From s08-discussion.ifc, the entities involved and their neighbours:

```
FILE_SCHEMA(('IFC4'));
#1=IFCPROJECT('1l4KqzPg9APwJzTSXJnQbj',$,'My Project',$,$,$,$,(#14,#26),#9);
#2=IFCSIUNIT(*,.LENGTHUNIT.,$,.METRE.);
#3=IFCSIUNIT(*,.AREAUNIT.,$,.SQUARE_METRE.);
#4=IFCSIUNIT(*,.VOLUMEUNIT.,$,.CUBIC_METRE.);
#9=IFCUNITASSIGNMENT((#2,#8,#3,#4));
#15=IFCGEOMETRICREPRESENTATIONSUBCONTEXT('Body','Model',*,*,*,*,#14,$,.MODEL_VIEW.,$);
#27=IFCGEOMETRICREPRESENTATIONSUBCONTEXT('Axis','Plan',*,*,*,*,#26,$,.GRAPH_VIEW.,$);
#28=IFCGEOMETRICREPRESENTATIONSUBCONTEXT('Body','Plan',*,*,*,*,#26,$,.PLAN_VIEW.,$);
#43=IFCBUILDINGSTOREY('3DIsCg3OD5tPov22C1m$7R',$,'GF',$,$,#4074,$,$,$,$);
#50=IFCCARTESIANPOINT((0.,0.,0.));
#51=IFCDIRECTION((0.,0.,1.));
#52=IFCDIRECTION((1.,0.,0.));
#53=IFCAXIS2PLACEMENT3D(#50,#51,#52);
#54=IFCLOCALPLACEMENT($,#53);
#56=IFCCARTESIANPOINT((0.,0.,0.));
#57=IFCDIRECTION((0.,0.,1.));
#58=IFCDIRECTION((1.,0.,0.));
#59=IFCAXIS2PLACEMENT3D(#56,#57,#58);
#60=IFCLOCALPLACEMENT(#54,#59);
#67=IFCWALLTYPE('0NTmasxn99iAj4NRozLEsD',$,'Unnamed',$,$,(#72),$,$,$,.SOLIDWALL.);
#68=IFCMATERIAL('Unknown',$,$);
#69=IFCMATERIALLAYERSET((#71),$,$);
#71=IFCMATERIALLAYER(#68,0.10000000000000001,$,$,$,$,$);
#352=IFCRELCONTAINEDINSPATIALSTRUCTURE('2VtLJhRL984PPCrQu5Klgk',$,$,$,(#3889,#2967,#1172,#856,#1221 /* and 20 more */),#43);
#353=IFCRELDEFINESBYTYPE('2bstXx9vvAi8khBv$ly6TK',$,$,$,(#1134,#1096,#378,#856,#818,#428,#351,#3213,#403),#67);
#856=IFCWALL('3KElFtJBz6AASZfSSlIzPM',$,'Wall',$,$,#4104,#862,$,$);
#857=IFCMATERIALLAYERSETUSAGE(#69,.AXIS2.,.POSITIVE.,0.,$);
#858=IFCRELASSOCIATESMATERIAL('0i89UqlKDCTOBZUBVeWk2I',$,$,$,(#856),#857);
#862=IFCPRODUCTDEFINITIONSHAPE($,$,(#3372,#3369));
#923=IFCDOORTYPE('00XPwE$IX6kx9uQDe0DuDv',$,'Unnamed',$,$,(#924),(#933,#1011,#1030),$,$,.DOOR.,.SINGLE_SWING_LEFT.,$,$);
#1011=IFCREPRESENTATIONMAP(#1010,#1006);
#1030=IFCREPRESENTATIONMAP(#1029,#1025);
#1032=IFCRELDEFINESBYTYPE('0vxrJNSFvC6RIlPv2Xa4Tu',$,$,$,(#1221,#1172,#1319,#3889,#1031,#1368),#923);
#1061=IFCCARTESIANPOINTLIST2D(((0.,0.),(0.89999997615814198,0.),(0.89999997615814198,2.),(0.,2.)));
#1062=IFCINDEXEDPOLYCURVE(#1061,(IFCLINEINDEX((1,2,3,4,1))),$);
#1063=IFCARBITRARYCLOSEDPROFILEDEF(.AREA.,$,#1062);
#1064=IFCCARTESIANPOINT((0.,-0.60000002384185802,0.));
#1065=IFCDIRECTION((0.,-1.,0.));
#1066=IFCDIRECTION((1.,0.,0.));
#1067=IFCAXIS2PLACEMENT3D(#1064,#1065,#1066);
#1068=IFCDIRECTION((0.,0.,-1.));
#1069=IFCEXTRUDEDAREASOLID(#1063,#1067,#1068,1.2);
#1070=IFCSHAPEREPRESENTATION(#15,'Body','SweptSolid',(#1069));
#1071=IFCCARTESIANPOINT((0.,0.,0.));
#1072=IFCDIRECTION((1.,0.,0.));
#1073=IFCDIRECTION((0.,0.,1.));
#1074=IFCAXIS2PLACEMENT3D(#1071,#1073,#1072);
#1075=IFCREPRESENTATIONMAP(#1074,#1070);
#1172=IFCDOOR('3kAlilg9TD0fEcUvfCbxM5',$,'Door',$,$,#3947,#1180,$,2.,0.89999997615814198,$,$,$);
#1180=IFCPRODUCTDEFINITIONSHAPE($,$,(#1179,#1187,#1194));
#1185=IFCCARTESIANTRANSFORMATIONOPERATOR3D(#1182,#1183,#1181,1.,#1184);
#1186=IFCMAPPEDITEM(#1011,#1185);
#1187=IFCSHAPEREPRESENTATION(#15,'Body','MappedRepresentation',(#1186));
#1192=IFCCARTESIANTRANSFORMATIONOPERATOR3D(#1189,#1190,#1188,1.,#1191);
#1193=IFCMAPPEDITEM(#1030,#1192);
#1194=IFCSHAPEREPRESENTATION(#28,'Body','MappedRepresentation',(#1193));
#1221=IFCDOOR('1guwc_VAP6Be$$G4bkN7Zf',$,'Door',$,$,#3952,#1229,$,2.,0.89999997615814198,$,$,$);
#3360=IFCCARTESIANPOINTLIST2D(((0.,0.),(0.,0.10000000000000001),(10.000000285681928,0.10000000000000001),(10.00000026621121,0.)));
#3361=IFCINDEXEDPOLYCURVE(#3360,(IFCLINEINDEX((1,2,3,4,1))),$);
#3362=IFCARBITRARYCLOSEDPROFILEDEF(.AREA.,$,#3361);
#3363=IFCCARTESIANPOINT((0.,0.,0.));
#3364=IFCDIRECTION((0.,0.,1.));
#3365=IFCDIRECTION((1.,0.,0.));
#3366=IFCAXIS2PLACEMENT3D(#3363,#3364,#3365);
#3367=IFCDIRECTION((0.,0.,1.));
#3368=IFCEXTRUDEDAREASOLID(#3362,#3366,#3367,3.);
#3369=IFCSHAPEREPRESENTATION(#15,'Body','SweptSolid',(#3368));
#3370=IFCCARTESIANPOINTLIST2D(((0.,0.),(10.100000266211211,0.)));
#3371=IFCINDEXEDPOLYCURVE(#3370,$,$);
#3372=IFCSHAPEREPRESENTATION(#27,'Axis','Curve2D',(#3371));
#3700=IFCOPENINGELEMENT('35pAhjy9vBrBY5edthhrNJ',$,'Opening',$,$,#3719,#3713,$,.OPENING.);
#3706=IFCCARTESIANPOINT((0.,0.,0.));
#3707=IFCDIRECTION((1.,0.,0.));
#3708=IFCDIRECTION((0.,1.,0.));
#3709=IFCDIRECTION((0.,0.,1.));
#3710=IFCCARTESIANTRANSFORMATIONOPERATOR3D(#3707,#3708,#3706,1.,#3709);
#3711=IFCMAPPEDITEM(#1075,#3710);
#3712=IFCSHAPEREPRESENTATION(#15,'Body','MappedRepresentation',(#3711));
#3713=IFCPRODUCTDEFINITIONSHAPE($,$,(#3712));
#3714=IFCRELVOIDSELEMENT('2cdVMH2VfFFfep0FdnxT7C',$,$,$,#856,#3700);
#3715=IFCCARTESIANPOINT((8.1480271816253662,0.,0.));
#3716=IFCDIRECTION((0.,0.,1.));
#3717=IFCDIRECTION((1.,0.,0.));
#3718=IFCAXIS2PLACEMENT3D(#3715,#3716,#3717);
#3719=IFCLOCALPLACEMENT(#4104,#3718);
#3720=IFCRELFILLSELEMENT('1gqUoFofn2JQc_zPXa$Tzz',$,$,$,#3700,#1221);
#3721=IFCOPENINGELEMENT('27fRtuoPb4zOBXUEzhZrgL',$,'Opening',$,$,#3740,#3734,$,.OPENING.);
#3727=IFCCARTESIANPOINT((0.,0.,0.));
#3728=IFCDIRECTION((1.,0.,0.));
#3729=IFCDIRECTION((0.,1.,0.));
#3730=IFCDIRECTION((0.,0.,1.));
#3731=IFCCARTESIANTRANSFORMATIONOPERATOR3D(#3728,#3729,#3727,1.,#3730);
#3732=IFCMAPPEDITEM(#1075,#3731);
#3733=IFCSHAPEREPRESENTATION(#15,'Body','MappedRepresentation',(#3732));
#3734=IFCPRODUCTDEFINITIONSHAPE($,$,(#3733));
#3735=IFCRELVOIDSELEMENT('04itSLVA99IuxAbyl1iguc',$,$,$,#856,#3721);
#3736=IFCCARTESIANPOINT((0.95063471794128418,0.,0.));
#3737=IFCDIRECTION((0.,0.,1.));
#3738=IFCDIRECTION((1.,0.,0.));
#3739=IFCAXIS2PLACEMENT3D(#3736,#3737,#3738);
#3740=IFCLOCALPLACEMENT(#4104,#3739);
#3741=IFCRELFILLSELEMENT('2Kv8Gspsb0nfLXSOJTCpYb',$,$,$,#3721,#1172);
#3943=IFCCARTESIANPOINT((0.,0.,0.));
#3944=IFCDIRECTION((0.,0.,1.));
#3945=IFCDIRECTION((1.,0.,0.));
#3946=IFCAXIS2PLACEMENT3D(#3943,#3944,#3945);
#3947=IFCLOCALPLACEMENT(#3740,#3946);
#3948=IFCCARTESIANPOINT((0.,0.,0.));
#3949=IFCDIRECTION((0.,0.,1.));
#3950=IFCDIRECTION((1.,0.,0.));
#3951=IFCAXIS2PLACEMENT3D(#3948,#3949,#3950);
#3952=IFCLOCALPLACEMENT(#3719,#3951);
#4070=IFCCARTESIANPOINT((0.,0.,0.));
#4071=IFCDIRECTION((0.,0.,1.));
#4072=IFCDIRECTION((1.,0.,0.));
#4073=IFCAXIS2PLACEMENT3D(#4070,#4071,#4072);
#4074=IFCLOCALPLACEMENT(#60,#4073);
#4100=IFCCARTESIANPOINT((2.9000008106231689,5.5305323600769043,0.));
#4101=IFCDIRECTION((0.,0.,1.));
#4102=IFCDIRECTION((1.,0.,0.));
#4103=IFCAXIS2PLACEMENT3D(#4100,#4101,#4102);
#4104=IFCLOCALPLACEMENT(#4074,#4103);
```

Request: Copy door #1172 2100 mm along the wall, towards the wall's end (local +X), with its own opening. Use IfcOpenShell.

```python
import ifcopenshell
import ifcopenshell.api.feature
import ifcopenshell.api.geometry
import ifcopenshell.api.root
import ifcopenshell.geom
import ifcopenshell.util.element
import ifcopenshell.util.placement
import ifcopenshell.util.shape

model = ifcopenshell.open("s08-discussion.ifc")
settings = ifcopenshell.geom.settings()


def volume(element):
    """Net volume in cubic metres, openings subtracted."""
    shape = ifcopenshell.geom.create_shape(settings, element)
    return ifcopenshell.util.shape.get_volume(shape.geometry)


door = model.by_id(1172)
opening = door.FillsVoids[0].RelatingOpeningElement
wall = opening.VoidsElements[0].RelatingBuildingElement
before = volume(wall)
shift = ifcopenshell.util.placement.get_local_placement(wall.ObjectPlacement)[:3, 0] * 2.1

# copy_class copies the void relationship, type, container and properties, but no geometry.
new_opening = ifcopenshell.api.root.copy_class(model, product=opening)
new_opening.Representation = ifcopenshell.util.element.copy_deep(
    model, opening.Representation, exclude=["IfcGeometricRepresentationContext", "IfcRepresentationMap"]
)
new_door = ifcopenshell.api.root.copy_class(model, product=door)
new_door.Representation = ifcopenshell.util.element.copy_deep(
    model, door.Representation, exclude=["IfcGeometricRepresentationContext", "IfcRepresentationMap"]
)
ifcopenshell.api.feature.add_filling(model, opening=new_opening, element=new_door)

for old, new in ((opening, new_opening), (door, new_door)):
    matrix = ifcopenshell.util.placement.get_local_placement(old.ObjectPlacement)
    matrix[:3, 3] += shift
    ifcopenshell.api.geometry.edit_object_placement(model, product=new, matrix=matrix, is_si=False)

after = volume(wall)

print(f"wall volume {before:.3f} -> {after:.3f} m3")

model.write("s08-discussion_v2.ifc")
```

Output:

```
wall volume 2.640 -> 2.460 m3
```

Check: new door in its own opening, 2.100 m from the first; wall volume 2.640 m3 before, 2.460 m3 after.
